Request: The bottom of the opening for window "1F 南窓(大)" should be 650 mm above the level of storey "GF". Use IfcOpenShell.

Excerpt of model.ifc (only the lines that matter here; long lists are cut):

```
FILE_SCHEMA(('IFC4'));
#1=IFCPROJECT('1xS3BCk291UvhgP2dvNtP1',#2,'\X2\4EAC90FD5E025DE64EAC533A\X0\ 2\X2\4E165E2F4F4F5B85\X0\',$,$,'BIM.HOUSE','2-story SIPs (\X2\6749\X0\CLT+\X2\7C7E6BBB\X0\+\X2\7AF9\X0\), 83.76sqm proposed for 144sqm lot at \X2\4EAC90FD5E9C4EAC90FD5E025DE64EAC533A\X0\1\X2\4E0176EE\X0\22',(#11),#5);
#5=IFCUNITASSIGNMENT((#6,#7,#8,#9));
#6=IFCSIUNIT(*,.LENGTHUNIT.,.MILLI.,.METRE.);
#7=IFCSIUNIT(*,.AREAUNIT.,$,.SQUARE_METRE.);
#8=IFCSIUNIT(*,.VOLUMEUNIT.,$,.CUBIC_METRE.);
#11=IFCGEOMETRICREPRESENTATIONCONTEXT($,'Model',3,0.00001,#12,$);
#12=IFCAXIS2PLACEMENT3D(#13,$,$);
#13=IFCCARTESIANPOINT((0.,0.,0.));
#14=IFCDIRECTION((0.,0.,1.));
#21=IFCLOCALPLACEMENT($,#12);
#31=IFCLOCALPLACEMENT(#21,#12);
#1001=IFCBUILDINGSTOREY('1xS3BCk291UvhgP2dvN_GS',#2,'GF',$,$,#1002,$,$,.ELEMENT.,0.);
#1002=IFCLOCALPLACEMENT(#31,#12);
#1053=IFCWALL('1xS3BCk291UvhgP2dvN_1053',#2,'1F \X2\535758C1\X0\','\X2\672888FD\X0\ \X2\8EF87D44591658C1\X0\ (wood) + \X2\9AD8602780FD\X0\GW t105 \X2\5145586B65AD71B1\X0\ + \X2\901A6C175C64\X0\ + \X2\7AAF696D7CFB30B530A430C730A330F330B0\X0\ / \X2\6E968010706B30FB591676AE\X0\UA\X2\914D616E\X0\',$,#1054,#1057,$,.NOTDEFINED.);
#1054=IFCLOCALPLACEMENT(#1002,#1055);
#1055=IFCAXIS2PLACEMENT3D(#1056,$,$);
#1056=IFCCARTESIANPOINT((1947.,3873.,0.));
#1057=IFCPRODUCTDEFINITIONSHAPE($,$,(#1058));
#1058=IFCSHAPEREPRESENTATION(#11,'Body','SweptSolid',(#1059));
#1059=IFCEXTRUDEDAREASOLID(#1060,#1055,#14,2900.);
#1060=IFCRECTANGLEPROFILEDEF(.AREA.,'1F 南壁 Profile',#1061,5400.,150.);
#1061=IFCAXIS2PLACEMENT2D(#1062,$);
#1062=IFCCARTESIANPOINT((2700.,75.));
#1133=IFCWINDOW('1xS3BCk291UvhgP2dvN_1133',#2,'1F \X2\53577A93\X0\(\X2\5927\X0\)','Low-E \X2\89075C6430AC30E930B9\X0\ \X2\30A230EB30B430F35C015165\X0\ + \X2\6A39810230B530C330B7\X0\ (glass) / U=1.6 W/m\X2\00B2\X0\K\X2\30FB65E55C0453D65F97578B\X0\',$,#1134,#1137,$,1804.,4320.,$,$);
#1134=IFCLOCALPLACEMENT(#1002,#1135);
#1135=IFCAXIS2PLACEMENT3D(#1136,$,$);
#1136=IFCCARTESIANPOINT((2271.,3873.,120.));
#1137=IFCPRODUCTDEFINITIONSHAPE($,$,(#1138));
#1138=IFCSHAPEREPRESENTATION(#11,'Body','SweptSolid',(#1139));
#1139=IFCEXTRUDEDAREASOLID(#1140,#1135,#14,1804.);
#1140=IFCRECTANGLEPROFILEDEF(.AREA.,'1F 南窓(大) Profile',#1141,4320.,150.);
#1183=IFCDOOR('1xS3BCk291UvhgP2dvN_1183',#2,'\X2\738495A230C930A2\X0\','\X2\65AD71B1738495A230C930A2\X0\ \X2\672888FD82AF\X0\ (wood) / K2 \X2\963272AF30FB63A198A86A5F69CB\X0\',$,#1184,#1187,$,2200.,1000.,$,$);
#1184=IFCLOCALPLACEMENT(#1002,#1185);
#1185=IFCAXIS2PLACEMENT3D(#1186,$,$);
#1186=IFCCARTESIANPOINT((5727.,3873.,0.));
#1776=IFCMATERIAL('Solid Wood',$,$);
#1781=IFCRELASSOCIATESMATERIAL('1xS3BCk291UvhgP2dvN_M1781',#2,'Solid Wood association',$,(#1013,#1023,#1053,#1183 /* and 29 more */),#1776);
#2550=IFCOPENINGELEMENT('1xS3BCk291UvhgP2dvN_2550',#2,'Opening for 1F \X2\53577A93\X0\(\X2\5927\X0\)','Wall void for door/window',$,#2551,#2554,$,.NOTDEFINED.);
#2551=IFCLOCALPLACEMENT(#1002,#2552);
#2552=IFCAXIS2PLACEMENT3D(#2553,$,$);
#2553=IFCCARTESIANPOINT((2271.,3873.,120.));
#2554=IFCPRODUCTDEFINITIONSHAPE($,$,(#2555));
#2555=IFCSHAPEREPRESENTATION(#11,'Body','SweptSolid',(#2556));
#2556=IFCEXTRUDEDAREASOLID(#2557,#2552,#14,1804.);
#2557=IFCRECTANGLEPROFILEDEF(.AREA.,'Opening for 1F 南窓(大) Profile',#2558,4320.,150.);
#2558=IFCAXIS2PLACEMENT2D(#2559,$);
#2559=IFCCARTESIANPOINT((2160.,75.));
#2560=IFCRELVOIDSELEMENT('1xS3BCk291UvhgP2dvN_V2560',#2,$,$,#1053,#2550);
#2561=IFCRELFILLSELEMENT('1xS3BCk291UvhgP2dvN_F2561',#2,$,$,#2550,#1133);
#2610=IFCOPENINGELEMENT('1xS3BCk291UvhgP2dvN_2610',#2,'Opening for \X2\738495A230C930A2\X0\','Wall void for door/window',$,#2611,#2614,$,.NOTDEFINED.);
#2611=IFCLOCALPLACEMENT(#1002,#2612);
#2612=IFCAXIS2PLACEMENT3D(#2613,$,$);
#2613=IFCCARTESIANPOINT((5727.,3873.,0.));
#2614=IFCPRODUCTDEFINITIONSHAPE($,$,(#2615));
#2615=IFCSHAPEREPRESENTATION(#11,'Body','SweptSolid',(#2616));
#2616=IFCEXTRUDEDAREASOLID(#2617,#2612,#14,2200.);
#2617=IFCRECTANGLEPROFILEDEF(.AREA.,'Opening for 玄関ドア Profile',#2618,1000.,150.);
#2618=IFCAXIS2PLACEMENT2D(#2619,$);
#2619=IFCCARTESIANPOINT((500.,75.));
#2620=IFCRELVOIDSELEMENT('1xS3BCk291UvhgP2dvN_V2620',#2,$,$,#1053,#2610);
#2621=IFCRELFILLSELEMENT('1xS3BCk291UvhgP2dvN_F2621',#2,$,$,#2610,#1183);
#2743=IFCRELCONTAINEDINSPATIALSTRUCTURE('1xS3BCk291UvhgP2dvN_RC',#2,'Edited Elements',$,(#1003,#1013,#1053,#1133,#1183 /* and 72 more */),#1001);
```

```python
import numpy as np
import ifcopenshell
import ifcopenshell.api.geometry
import ifcopenshell.geom
import ifcopenshell.util.element
import ifcopenshell.util.placement
import ifcopenshell.util.shape
import ifcopenshell.util.unit

model = ifcopenshell.open("model.ifc")
unit_scale = ifcopenshell.util.unit.calculate_unit_scale(model)

window = model.by_guid("1xS3BCk291UvhgP2dvN_1133")
opening = window.FillsVoids[0].RelatingOpeningElement
storey = ifcopenshell.util.element.get_container(window, ifc_class="IfcBuildingStorey")
level = ifcopenshell.util.placement.get_local_placement(storey.ObjectPlacement)[2, 3]

# The opening's origin need not be at the sill, so measure its lowest point.
shape = ifcopenshell.geom.create_shape(ifcopenshell.geom.settings(), opening)
bottom = ifcopenshell.util.shape.get_shape_bottom_elevation(shape, shape.geometry) / unit_scale
dz = level + 0.65 / unit_scale - bottom

shift = np.array([0.0, 0.0, dz])
# The window is not placed relative to its opening, so move both.
for product in (opening, window):
    matrix = ifcopenshell.util.placement.get_local_placement(product.ObjectPlacement)
    matrix[:3, 3] += shift
    ifcopenshell.api.geometry.edit_object_placement(model, product=product, matrix=matrix, is_si=False)

print(f"moved by {dz * unit_scale:+.3f} m")

model.write("model_updated.ifc")
```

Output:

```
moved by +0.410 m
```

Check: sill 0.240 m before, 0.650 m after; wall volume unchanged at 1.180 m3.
